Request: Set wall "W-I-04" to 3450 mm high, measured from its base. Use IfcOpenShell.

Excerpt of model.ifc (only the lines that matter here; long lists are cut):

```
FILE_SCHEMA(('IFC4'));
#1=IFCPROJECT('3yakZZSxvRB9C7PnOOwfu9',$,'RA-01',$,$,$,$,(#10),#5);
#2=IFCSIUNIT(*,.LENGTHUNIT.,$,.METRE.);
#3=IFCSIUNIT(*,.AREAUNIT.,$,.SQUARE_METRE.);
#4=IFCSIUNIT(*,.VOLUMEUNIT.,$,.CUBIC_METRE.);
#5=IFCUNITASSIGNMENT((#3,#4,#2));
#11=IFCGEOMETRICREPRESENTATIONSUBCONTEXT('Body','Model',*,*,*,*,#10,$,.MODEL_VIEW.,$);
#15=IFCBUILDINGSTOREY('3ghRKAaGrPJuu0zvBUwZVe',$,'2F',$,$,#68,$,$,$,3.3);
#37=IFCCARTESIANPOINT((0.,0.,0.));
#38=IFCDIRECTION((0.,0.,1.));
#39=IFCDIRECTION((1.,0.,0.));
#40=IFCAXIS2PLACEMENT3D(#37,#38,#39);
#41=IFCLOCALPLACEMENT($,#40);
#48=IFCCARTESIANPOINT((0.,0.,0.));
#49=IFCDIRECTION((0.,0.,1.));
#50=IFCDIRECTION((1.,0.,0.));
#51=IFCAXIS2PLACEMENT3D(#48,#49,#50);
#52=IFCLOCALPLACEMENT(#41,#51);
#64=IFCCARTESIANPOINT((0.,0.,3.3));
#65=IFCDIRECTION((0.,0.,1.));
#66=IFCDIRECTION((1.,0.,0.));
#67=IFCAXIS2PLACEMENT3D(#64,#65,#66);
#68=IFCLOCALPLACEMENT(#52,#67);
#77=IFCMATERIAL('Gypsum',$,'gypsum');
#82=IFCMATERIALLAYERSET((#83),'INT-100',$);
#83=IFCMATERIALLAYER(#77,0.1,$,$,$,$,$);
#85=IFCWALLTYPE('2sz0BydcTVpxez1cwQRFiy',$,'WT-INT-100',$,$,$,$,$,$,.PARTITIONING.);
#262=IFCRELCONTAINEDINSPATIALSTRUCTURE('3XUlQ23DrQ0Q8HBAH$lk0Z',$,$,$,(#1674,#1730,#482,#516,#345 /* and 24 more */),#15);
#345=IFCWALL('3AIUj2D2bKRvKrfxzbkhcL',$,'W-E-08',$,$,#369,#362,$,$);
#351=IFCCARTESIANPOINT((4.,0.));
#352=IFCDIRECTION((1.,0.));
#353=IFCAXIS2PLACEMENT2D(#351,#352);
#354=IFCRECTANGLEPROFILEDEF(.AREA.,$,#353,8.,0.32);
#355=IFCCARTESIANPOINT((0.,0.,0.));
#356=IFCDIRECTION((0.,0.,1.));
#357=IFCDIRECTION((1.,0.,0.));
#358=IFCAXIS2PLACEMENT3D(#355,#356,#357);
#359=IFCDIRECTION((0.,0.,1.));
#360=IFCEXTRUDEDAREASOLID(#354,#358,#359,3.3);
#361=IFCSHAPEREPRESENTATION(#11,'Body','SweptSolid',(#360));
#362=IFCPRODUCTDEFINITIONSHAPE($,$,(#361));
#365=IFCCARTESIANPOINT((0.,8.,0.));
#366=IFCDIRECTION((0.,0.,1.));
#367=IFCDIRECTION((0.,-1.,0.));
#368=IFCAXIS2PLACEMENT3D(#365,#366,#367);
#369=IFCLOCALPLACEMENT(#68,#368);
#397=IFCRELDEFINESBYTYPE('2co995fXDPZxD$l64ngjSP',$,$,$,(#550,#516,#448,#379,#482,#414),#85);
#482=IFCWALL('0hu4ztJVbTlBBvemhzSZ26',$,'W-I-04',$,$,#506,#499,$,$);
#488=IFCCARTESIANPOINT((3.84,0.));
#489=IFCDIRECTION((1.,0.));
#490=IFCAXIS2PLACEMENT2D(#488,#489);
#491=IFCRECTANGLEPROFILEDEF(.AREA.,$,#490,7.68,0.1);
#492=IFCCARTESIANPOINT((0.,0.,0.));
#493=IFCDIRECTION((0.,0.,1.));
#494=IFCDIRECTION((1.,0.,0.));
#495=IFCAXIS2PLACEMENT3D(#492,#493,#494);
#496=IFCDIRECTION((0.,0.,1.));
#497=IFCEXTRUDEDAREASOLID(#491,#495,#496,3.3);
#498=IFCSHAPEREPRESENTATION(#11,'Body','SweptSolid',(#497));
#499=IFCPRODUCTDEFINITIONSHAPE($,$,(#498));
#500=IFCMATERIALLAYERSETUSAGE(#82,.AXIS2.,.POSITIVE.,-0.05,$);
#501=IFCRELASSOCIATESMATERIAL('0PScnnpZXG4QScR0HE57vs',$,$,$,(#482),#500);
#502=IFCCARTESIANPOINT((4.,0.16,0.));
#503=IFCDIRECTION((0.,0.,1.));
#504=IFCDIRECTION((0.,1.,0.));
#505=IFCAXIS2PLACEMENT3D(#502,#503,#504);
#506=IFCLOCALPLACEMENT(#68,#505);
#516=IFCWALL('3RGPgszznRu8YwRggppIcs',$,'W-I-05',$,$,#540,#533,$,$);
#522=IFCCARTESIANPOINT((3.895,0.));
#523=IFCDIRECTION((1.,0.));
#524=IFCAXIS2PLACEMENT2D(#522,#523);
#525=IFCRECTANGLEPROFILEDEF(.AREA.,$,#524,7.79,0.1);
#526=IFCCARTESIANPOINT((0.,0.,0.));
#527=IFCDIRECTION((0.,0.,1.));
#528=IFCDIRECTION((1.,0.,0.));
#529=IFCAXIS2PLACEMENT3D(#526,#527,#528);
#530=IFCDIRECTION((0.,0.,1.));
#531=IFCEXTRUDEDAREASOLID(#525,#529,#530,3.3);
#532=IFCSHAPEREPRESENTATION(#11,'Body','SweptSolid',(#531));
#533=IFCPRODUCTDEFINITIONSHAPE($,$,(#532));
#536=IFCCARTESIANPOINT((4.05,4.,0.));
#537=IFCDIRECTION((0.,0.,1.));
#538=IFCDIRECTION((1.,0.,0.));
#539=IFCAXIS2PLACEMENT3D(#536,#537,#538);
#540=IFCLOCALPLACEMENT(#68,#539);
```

```python
import ifcopenshell
import ifcopenshell.geom
import ifcopenshell.util.representation
import ifcopenshell.util.shape
import ifcopenshell.util.unit

model = ifcopenshell.open("model.ifc")
unit_scale = ifcopenshell.util.unit.calculate_unit_scale(model)
settings = ifcopenshell.geom.settings()


def volume(element):
    """Net volume in cubic metres, openings subtracted."""
    shape = ifcopenshell.geom.create_shape(settings, element)
    return ifcopenshell.util.shape.get_volume(shape.geometry)


wall = model.by_guid("0hu4ztJVbTlBBvemhzSZ26")
before = volume(wall)

body = ifcopenshell.util.representation.get_representation(wall, "Model", "Body")
solid = body.Items[0]
old_height = solid.Depth
solid.Depth = 3.45 / unit_scale
after = volume(wall)

print(f"height {old_height:g} -> {solid.Depth:g}, volume {before:.3f} -> {after:.3f} m3")

model.write("model_updated.ifc")
```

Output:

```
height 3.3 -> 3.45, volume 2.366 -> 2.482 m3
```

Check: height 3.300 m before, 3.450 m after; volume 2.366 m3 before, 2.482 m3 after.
